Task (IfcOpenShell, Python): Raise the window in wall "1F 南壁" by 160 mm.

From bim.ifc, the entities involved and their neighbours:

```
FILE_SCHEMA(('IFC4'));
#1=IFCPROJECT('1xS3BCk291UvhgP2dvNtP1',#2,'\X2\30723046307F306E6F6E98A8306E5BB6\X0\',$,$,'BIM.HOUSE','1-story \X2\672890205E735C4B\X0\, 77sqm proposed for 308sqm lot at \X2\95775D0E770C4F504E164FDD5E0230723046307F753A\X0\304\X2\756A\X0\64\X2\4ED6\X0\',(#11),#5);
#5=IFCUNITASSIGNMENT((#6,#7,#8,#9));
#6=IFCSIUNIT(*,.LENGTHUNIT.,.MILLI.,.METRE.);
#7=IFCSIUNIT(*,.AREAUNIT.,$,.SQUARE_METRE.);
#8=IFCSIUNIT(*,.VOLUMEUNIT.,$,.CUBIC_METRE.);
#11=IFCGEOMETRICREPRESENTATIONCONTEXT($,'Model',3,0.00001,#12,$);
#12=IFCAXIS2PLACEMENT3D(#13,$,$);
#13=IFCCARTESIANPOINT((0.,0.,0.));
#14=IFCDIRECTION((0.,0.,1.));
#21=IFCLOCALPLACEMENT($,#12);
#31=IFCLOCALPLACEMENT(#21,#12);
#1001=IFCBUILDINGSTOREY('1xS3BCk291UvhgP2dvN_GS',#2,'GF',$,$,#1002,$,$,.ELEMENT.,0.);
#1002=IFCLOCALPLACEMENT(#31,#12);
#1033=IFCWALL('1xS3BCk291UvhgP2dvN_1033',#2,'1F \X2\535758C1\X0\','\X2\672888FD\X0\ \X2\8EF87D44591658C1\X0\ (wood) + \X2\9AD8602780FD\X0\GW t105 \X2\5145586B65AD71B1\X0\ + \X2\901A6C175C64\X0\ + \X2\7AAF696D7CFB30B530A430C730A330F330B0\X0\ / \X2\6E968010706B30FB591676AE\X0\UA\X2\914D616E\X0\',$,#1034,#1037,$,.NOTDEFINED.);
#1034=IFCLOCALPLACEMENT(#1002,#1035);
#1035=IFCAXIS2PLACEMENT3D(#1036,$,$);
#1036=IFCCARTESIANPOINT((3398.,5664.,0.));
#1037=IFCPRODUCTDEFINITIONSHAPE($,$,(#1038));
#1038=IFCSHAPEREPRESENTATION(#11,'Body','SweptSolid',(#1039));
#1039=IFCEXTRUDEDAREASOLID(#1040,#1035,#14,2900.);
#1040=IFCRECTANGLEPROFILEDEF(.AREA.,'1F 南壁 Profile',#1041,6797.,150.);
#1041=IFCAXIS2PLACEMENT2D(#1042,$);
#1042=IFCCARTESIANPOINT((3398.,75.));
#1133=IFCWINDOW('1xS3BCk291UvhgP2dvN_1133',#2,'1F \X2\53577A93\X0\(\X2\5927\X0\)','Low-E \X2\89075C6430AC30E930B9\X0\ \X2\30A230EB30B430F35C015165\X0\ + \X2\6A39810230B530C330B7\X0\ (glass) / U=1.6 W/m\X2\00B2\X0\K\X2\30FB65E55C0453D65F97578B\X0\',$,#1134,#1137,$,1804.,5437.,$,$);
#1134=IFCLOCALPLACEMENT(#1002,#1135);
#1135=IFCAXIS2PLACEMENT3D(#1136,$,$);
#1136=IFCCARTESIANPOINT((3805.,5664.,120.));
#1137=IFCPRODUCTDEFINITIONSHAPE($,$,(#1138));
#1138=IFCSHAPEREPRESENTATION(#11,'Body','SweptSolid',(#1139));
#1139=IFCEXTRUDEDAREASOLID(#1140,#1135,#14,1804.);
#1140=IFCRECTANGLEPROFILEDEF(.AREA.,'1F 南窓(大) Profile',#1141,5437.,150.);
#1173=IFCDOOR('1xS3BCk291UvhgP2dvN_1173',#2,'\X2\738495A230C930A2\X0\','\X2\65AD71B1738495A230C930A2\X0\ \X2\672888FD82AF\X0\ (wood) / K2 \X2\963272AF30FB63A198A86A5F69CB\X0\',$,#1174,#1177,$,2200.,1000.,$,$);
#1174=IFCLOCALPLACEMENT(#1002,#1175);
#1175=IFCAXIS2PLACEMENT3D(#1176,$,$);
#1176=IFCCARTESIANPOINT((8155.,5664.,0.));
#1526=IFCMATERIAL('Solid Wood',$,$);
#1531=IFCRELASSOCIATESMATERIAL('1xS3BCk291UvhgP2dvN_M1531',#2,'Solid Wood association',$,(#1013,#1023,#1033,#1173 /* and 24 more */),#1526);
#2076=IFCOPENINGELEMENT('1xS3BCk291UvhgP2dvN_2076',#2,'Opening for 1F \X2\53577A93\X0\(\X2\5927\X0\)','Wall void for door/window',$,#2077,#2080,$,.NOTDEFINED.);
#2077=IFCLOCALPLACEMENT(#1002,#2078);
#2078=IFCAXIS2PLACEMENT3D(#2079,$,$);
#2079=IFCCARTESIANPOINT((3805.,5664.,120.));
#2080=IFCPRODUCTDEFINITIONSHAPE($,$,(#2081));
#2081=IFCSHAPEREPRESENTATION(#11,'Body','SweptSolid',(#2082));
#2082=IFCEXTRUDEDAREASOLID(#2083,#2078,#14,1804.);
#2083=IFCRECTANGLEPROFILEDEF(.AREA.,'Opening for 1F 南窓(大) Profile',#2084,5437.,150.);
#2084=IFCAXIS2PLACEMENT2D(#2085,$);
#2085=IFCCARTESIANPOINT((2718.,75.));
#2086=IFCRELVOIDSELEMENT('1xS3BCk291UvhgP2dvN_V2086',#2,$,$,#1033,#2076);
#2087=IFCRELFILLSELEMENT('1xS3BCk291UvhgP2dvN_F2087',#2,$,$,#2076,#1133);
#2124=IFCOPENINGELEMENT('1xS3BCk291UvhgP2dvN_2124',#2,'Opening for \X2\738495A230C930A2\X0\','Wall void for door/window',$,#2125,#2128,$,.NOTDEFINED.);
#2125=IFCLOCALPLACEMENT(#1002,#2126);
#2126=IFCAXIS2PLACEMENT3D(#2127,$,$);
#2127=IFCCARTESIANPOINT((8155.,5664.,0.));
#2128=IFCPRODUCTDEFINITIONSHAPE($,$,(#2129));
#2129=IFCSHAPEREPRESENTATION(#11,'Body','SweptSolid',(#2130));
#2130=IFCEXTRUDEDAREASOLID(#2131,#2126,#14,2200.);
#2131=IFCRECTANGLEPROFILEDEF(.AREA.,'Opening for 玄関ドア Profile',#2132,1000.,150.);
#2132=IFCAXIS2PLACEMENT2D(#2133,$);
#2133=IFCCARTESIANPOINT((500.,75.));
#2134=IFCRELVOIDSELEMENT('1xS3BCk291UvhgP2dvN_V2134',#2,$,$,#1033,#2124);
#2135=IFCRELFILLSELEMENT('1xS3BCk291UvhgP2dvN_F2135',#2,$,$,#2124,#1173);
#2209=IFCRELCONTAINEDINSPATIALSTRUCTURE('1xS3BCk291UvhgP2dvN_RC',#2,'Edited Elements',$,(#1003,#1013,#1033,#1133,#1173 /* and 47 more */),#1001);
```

```python
import numpy as np
import ifcopenshell
import ifcopenshell.api.geometry
import ifcopenshell.util.placement
import ifcopenshell.util.unit

model = ifcopenshell.open("bim.ifc")
unit_scale = ifcopenshell.util.unit.calculate_unit_scale(model)

window = model.by_guid("1xS3BCk291UvhgP2dvN_1133")
opening = window.FillsVoids[0].RelatingOpeningElement
dz = 160.0

shift = np.array([0.0, 0.0, dz])
# The window is not placed relative to its opening, so move both.
for product in (opening, window):
    matrix = ifcopenshell.util.placement.get_local_placement(product.ObjectPlacement)
    matrix[:3, 3] += shift
    ifcopenshell.api.geometry.edit_object_placement(model, product=product, matrix=matrix, is_si=False)

print(f"moved by {dz * unit_scale:+.3f} m")

model.write("bim_rev.ifc")
```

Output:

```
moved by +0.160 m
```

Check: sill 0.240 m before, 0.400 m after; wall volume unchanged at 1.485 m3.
